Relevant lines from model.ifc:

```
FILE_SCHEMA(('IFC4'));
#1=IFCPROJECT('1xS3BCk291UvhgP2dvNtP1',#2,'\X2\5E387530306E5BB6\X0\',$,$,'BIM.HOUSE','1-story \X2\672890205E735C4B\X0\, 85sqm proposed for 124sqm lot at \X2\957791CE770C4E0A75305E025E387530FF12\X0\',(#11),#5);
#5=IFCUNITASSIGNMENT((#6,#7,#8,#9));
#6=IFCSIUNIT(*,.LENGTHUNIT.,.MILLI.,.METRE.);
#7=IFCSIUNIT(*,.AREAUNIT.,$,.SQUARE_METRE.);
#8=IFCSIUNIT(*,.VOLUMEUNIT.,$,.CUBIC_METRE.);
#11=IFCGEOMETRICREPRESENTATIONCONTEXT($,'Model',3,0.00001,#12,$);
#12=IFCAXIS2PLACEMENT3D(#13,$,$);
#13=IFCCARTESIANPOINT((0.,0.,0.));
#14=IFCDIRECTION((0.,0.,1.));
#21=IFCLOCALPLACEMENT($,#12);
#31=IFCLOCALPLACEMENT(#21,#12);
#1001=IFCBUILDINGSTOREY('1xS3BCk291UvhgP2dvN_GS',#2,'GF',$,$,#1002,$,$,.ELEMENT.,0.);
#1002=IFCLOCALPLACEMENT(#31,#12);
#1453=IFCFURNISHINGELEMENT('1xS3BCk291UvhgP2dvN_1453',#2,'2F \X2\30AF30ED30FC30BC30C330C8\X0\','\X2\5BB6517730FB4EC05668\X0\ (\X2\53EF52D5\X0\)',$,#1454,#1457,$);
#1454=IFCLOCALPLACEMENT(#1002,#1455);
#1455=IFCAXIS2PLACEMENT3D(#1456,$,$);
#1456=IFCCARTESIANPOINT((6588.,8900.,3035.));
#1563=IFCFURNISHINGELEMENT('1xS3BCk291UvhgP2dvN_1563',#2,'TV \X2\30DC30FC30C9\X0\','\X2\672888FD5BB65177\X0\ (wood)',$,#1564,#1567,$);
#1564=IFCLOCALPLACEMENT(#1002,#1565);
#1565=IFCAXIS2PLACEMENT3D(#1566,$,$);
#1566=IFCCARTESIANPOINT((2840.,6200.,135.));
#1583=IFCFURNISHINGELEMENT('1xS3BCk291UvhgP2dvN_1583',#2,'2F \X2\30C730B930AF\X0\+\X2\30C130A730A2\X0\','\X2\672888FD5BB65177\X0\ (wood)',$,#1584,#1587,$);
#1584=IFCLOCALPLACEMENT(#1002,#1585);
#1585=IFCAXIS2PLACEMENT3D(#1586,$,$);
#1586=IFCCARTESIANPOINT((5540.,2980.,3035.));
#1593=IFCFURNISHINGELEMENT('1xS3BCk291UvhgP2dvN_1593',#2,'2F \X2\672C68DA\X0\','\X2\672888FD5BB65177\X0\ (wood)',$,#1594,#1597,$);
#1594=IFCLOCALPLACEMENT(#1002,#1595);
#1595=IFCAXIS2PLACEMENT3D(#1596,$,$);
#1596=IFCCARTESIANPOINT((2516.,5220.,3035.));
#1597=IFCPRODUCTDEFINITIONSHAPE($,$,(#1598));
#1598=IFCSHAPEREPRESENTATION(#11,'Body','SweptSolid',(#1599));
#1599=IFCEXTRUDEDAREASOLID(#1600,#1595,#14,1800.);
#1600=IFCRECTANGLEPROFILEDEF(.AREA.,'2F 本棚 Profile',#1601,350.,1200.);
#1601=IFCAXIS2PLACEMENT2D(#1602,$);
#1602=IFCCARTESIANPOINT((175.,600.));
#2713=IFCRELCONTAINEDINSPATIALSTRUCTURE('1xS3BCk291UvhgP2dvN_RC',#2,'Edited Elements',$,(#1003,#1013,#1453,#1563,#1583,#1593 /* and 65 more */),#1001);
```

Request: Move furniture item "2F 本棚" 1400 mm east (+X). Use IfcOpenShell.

```python
import ifcopenshell
import ifcopenshell.api.geometry
import ifcopenshell.util.placement

model = ifcopenshell.open("model.ifc")

item = model.by_id(1593)
matrix = ifcopenshell.util.placement.get_local_placement(item.ObjectPlacement)
matrix[0, 3] += 1400.0
ifcopenshell.api.geometry.edit_object_placement(model, product=item, matrix=matrix, is_si=False)

print(ifcopenshell.util.placement.get_local_placement(item.ObjectPlacement).round(3) + 0.0)

model.write("model_edited.ifc")
```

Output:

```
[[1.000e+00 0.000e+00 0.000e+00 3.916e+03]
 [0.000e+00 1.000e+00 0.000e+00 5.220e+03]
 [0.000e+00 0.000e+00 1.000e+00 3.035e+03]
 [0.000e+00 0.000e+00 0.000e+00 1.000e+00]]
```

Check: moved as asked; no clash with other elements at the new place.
